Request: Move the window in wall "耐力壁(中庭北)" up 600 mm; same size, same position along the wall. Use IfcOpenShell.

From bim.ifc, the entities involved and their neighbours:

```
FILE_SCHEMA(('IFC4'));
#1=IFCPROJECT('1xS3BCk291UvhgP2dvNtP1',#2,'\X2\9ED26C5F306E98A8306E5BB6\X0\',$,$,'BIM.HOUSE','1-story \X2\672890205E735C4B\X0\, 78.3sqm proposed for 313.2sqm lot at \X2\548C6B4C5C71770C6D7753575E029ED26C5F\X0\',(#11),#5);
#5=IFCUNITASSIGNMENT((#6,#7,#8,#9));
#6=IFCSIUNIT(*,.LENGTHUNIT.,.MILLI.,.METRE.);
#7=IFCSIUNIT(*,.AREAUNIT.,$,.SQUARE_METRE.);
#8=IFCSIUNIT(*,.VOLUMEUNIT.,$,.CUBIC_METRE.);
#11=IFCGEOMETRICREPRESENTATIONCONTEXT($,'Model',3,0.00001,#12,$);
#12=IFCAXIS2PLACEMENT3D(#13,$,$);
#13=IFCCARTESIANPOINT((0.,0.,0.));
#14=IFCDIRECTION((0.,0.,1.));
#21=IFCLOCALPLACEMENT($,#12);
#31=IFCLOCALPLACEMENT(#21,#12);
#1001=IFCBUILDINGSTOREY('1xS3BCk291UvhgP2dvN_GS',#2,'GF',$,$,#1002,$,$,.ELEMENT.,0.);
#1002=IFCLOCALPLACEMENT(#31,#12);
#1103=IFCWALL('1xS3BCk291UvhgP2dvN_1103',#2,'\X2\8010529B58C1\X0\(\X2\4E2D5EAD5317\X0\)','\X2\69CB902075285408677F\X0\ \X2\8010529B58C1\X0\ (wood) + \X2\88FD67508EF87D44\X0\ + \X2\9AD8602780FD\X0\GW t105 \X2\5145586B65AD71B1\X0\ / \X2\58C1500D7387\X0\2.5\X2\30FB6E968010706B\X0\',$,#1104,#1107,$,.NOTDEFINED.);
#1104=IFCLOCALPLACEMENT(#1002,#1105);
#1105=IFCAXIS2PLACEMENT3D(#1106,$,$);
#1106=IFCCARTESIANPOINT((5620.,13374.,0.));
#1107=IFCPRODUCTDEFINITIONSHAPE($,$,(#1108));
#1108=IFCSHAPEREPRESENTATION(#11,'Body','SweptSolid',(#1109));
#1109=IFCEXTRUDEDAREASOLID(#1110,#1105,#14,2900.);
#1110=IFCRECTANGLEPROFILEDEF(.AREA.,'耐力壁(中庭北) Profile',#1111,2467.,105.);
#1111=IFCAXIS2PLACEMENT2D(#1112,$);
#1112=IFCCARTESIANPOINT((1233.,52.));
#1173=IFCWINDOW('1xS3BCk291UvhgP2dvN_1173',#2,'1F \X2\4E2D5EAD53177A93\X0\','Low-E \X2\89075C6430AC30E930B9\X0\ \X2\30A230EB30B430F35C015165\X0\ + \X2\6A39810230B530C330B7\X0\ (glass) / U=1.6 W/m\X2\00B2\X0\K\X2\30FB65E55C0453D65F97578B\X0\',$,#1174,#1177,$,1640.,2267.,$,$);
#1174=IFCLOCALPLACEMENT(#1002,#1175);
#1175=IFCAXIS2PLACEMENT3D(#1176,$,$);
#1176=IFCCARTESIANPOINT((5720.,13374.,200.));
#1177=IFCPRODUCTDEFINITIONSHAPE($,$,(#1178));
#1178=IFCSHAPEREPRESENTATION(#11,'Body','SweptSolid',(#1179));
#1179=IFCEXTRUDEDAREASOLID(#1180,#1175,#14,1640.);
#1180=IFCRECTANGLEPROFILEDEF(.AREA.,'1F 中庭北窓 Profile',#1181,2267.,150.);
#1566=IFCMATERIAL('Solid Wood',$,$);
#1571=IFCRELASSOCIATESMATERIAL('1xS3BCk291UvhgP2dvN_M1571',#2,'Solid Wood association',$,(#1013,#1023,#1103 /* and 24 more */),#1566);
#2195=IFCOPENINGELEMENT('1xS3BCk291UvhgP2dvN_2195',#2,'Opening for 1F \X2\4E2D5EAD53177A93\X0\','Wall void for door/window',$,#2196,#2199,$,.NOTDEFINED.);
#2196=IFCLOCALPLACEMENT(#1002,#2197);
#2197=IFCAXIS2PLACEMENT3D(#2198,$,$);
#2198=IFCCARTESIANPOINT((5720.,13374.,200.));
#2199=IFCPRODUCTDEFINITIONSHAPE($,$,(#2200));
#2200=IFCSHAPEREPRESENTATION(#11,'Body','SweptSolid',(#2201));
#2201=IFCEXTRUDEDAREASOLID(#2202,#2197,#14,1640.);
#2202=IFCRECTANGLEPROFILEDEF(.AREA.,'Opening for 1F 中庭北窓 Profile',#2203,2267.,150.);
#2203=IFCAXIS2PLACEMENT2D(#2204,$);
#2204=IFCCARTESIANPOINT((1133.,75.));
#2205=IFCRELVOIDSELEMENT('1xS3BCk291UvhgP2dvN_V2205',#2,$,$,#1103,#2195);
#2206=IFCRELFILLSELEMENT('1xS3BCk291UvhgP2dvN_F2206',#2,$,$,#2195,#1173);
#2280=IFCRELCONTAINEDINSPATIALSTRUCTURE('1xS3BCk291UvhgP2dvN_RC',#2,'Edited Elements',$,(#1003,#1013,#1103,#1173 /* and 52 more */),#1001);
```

```python
import numpy as np
import ifcopenshell
import ifcopenshell.api.geometry
import ifcopenshell.util.placement
import ifcopenshell.util.unit

model = ifcopenshell.open("bim.ifc")
unit_scale = ifcopenshell.util.unit.calculate_unit_scale(model)

window = model.by_guid("1xS3BCk291UvhgP2dvN_1173")
opening = window.FillsVoids[0].RelatingOpeningElement
dz = 600.0

shift = np.array([0.0, 0.0, dz])
# The window is not placed relative to its opening, so move both.
for product in (opening, window):
    matrix = ifcopenshell.util.placement.get_local_placement(product.ObjectPlacement)
    matrix[:3, 3] += shift
    ifcopenshell.api.geometry.edit_object_placement(model, product=product, matrix=matrix, is_si=False)

print(f"moved by {dz * unit_scale:+.3f} m")

model.write("bim_v2.ifc")
```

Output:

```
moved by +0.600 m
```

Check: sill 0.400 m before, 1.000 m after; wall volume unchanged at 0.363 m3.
